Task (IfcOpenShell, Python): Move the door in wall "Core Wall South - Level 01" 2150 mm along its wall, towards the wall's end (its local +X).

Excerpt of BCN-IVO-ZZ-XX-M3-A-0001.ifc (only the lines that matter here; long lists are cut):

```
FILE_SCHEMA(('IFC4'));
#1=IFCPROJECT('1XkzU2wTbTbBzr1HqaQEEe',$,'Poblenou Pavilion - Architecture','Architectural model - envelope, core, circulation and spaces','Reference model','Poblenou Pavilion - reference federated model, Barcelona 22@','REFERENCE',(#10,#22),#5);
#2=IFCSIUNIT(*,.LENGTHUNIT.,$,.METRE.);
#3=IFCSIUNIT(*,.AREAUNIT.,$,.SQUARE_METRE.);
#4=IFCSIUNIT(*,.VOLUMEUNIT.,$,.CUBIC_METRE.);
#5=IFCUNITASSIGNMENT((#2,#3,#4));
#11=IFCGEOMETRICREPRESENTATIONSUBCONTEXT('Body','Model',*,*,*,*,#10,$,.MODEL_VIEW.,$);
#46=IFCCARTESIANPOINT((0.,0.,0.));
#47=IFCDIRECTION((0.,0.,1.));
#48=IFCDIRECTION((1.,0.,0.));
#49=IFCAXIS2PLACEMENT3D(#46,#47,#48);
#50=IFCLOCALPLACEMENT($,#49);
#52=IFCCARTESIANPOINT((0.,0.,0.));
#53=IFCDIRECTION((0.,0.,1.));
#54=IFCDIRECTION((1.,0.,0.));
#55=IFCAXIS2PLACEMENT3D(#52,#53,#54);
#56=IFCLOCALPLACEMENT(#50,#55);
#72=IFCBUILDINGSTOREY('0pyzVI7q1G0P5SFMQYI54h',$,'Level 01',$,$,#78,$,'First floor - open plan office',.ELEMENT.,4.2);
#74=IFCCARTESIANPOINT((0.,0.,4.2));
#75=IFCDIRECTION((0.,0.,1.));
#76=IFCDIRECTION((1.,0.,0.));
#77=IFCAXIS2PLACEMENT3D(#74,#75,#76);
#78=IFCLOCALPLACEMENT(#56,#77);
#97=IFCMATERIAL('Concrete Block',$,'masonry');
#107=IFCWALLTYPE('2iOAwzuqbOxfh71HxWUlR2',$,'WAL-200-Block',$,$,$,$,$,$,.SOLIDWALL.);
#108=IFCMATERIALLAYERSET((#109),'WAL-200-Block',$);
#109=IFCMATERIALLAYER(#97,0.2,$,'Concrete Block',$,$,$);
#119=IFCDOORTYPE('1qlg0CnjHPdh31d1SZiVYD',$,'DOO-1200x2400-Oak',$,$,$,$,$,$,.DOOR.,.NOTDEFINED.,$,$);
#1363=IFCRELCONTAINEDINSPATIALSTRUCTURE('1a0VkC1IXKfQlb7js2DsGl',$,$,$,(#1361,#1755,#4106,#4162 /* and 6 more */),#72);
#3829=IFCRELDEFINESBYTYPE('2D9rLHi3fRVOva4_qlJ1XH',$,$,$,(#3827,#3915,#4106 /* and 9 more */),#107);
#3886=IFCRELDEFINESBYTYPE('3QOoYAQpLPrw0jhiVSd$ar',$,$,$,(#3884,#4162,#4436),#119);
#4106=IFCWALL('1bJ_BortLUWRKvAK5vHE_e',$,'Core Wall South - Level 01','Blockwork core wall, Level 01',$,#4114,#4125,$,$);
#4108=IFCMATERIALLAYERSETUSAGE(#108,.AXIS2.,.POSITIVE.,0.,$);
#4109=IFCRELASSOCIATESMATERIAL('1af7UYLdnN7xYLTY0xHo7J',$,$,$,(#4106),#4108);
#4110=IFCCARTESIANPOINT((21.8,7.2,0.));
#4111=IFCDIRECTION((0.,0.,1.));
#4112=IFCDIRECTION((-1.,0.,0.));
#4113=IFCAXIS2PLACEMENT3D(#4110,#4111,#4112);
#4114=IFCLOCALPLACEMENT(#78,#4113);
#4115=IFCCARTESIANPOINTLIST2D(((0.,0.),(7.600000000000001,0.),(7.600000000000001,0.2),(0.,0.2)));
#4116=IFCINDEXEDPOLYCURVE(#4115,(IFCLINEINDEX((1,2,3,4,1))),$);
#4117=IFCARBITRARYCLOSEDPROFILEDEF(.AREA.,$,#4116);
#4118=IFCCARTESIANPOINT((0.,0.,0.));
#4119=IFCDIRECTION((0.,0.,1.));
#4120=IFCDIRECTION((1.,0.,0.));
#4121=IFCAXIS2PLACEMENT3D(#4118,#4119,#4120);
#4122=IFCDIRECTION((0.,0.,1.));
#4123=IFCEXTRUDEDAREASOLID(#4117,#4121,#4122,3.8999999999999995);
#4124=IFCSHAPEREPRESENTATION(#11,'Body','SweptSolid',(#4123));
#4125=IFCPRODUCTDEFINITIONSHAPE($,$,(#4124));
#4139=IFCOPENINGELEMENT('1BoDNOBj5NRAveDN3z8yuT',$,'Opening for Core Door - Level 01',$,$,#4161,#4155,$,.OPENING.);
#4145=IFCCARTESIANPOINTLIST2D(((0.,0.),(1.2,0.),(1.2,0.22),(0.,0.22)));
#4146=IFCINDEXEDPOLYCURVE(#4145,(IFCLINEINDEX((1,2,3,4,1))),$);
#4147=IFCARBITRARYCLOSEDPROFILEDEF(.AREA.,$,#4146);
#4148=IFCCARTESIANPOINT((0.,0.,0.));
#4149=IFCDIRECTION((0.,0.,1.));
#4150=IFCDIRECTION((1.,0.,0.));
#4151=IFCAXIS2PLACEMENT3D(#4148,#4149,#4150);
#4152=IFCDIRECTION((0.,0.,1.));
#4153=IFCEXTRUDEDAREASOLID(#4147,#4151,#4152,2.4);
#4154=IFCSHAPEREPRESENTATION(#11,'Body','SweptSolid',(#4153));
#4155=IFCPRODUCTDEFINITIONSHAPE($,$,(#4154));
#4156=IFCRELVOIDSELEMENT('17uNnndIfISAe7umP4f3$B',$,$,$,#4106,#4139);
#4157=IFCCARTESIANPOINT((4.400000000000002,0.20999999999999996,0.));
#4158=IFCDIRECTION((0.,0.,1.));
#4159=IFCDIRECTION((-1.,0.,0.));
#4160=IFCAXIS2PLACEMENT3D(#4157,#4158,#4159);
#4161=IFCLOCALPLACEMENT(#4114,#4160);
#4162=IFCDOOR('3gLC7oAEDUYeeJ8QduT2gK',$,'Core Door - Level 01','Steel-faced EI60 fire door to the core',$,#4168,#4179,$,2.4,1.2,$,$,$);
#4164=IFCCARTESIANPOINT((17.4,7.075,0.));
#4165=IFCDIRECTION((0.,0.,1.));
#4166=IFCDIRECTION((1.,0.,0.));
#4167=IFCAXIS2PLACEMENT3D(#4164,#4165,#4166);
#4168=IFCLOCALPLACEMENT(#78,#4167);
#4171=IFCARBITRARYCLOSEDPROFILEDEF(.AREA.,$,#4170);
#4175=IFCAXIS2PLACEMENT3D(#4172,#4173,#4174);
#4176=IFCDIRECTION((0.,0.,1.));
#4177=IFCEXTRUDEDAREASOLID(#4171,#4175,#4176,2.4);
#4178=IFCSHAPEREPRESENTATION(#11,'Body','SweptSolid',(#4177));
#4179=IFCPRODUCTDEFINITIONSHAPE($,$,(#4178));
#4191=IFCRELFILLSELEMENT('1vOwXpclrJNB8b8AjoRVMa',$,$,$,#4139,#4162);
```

```python
import ifcopenshell
import ifcopenshell.api.geometry
import ifcopenshell.util.placement

model = ifcopenshell.open("BCN-IVO-ZZ-XX-M3-A-0001.ifc")

door = model.by_guid("3gLC7oAEDUYeeJ8QduT2gK")
opening = door.FillsVoids[0].RelatingOpeningElement
wall = opening.VoidsElements[0].RelatingBuildingElement

wall_matrix = ifcopenshell.util.placement.get_local_placement(wall.ObjectPlacement)
shift = wall_matrix[:3, 0] * 2.15
before = ifcopenshell.util.placement.get_local_placement(door.ObjectPlacement)[:3, 3].copy()

# The door is not placed relative to its opening, so move both.
for product in (opening, door):
    matrix = ifcopenshell.util.placement.get_local_placement(product.ObjectPlacement)
    matrix[:3, 3] += shift
    ifcopenshell.api.geometry.edit_object_placement(model, product=product, matrix=matrix, is_si=False)

after = ifcopenshell.util.placement.get_local_placement(door.ObjectPlacement)[:3, 3]
print("door moved by", (after - before).round(3) + 0.0)

model.write("BCN-IVO-ZZ-XX-M3-A-0001-out.ifc")
```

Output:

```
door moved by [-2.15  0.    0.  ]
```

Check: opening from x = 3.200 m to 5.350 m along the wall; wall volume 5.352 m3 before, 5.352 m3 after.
